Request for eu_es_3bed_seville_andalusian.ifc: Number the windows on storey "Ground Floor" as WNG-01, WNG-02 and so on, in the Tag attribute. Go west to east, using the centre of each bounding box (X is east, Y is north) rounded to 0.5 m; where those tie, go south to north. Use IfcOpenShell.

First a look at what the model holds.

```python
import ifcopenshell
import ifcopenshell.util.element
import ifcopenshell.util.placement

model = ifcopenshell.open("eu_es_3bed_seville_andalusian.ifc")
print(model.schema)
storey = next(s for s in model.by_type("IfcBuildingStorey") if s.Name == "Ground Floor")
windows = [e for e in ifcopenshell.util.element.get_decomposition(storey) if e.is_a("IfcWindow")]
for e in sorted(windows, key=lambda e: e.id()):
    origin = ifcopenshell.util.placement.get_local_placement(e.ObjectPlacement)[:3, 3]
    print(e.id(), e.Tag, e.Name, origin.round(2) + 0.0, sep=" | ")
```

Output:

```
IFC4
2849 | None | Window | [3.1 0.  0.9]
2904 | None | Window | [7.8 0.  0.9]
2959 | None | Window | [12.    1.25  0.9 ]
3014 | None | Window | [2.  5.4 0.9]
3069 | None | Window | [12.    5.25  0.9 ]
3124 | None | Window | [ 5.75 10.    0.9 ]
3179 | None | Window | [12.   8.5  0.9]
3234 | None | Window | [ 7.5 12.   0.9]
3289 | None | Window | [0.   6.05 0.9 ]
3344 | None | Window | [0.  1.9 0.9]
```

```python
import ifcopenshell
import ifcopenshell.geom
import ifcopenshell.util.element
import ifcopenshell.util.shape

model = ifcopenshell.open("eu_es_3bed_seville_andalusian.ifc")
settings = ifcopenshell.geom.settings()
settings.set("use-world-coords", True)


def centre(element):
    shape = ifcopenshell.geom.create_shape(settings, element)
    return ifcopenshell.util.shape.get_bbox_centroid(shape.geometry)


storey = next(s for s in model.by_type("IfcBuildingStorey") if s.Name == "Ground Floor")
windows = [e for e in ifcopenshell.util.element.get_decomposition(storey) if e.is_a("IfcWindow")]

# Insertion points can sit at a corner or the storey origin, so sort by the geometry (in metres).
centres = {e: centre(e) for e in windows}
windows.sort(key=lambda e: (round(centres[e][0] / 0.5), centres[e][1]))

for i, e in enumerate(windows, start=1):
    number = f"WNG-{i:02d}"
    e.Tag = number
    print(e.id(), number)

model.write("eu_es_3bed_seville_andalusian_edited.ifc")
```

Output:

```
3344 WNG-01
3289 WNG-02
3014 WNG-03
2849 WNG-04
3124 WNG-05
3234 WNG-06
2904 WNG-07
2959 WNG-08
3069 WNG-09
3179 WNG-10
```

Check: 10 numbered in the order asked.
